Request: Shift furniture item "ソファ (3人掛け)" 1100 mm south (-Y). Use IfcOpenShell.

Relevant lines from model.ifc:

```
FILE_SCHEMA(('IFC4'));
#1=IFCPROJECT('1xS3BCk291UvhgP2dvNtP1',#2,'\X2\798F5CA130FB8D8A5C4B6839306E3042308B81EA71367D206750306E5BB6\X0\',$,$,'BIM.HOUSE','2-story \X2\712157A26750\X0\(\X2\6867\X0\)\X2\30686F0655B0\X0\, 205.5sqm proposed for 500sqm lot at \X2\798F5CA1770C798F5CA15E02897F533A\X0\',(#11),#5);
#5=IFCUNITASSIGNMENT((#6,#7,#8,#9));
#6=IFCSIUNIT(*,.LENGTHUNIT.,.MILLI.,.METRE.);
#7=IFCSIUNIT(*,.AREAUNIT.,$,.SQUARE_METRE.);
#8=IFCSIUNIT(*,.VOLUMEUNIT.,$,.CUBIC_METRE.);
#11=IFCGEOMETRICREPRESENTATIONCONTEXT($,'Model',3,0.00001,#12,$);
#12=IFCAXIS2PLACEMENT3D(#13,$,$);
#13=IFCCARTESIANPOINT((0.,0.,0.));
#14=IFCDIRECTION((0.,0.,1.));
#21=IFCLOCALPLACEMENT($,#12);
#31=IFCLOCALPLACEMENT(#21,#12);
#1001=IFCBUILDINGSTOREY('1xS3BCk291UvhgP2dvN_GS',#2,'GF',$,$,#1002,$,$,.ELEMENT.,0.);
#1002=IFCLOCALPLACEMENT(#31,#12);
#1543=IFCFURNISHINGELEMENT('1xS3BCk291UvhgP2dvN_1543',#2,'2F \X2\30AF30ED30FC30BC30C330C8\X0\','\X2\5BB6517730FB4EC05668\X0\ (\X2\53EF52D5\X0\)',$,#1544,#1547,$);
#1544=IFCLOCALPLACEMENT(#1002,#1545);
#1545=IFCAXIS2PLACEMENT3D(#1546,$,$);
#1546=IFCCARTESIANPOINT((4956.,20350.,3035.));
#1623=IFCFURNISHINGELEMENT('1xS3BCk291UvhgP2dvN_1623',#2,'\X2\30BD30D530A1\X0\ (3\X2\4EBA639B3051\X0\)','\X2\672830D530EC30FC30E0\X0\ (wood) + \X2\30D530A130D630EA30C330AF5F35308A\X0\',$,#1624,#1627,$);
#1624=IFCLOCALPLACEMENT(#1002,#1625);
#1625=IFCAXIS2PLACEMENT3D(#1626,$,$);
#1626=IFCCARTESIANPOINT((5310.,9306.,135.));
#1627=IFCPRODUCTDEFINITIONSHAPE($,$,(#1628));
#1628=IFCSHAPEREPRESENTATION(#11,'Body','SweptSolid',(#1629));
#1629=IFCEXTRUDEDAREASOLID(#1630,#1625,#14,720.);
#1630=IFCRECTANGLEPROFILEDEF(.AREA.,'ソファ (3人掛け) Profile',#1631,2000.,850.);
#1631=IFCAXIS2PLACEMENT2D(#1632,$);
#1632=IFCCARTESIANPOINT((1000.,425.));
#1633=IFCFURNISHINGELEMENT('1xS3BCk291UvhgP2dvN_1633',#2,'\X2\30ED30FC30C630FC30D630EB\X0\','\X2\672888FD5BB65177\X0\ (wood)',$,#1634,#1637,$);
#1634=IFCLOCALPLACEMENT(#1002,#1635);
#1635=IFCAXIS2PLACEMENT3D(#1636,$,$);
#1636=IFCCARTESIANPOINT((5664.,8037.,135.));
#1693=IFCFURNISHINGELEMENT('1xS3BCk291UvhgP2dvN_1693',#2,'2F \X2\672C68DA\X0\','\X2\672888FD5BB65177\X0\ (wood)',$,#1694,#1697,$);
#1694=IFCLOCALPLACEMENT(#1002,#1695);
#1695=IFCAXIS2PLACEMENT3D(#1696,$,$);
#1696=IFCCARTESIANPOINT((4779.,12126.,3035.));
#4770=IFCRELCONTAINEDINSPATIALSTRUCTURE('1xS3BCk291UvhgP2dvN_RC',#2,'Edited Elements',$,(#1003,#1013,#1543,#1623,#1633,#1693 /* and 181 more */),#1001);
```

```python
import ifcopenshell
import ifcopenshell.api.geometry
import ifcopenshell.util.placement
import ifcopenshell.util.unit

model = ifcopenshell.open("model.ifc")
unit_scale = ifcopenshell.util.unit.calculate_unit_scale(model)

item = model.by_guid("1xS3BCk291UvhgP2dvN_1623")
matrix = ifcopenshell.util.placement.get_local_placement(item.ObjectPlacement)
matrix[1, 3] -= 1.1 / unit_scale
ifcopenshell.api.geometry.edit_object_placement(model, product=item, matrix=matrix, is_si=False)

print(ifcopenshell.util.placement.get_local_placement(item.ObjectPlacement).round(3) + 0.0)

model.write("model_v2.ifc")
```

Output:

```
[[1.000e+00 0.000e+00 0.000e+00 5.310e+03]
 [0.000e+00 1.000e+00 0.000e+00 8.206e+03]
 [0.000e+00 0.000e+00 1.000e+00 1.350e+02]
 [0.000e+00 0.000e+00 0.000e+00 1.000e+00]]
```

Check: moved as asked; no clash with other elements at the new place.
